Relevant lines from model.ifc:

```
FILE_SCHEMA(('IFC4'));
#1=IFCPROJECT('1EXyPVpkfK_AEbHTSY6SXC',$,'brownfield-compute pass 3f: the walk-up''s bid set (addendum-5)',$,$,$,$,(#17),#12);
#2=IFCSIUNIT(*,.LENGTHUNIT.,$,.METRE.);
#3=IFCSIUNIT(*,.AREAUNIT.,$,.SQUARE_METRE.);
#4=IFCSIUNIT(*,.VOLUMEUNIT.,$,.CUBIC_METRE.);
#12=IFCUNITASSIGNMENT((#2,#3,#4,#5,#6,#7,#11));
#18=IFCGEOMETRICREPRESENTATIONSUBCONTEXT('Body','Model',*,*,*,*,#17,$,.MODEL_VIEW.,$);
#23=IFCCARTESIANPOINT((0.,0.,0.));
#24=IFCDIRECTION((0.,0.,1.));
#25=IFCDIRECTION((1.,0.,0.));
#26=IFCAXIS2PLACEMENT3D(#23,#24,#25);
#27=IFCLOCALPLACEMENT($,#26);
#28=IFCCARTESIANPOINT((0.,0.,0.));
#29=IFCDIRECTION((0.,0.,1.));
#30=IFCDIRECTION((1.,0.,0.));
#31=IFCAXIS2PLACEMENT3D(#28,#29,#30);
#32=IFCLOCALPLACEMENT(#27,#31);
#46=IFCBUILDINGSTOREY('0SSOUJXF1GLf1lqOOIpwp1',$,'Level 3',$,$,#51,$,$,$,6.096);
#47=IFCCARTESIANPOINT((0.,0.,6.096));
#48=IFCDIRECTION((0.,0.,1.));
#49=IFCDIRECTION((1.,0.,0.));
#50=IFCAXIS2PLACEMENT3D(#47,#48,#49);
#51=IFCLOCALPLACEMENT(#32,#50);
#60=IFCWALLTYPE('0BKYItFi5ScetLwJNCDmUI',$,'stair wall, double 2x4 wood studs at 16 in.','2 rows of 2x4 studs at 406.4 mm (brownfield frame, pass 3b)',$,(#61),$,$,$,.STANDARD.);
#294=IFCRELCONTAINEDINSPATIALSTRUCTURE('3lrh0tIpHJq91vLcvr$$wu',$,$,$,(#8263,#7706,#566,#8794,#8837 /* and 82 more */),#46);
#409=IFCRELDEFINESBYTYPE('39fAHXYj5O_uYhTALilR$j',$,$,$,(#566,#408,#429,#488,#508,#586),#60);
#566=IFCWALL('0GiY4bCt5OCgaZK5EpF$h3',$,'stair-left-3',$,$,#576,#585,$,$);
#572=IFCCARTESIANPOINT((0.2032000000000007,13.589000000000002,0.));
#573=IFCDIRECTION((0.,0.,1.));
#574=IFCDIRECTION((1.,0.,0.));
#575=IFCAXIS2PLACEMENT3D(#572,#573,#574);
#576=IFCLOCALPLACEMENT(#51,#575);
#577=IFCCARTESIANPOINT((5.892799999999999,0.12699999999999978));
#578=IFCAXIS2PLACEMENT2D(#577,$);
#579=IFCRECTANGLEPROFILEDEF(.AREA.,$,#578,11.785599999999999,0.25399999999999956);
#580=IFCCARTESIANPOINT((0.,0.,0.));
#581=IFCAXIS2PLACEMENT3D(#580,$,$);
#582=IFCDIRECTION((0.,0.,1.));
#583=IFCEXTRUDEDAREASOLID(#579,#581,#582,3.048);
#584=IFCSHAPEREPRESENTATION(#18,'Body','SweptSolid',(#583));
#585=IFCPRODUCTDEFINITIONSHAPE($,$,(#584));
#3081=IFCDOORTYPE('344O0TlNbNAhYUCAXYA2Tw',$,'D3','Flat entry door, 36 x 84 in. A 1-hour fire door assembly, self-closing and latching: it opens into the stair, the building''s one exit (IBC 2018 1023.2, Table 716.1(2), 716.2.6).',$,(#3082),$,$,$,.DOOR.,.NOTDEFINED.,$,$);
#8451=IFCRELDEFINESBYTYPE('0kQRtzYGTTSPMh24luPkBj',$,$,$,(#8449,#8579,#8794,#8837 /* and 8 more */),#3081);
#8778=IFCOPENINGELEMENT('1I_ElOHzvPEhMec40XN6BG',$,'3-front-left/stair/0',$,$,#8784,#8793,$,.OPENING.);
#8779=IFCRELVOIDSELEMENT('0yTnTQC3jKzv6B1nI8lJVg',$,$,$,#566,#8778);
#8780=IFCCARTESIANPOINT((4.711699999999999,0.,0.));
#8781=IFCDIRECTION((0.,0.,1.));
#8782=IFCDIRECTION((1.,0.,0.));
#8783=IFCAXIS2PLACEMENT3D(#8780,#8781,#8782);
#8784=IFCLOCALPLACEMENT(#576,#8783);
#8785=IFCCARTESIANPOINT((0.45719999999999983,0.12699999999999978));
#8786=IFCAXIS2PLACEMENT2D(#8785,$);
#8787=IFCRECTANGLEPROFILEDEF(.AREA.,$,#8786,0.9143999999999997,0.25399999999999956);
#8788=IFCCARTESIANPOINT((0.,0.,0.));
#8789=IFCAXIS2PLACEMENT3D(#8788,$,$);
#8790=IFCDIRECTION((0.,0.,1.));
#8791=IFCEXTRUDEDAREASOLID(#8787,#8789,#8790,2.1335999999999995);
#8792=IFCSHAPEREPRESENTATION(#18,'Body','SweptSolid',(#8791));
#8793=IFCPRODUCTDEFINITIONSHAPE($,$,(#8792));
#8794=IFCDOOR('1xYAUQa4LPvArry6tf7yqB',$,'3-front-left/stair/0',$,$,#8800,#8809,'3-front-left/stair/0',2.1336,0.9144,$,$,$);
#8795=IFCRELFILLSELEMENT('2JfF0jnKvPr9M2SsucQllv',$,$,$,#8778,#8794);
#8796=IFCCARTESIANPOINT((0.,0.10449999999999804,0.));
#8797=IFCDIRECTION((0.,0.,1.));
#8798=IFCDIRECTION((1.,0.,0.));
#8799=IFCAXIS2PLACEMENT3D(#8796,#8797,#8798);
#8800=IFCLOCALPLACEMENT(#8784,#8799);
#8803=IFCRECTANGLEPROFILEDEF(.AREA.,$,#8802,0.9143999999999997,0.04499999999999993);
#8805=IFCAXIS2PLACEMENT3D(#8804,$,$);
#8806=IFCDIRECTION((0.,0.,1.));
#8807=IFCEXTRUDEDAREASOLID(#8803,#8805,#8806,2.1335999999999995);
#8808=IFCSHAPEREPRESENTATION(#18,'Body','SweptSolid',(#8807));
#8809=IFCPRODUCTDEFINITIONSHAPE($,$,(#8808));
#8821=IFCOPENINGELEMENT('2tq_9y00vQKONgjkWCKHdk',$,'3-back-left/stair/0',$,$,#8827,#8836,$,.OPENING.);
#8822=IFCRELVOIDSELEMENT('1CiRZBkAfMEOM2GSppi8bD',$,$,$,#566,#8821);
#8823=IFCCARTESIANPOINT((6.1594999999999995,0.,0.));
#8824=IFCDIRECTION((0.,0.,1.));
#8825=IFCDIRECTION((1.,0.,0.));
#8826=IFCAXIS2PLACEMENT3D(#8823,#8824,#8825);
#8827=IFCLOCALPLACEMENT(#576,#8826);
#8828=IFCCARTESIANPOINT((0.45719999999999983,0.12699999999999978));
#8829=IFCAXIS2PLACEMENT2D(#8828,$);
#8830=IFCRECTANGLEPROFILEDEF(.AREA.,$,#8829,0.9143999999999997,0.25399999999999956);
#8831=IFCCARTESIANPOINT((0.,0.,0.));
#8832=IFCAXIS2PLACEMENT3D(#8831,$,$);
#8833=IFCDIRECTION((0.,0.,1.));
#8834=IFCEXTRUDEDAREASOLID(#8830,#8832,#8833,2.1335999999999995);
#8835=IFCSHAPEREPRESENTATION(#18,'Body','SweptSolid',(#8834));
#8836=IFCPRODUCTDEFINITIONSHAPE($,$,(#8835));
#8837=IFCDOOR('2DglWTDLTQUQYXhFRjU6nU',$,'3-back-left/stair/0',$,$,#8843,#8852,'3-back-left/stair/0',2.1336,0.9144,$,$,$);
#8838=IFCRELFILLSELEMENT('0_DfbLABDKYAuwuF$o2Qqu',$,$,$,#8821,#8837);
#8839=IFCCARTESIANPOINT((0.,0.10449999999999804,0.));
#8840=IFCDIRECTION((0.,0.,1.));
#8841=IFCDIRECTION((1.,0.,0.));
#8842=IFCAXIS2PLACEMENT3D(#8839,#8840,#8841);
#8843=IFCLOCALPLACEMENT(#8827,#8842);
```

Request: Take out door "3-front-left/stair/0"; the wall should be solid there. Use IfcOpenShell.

```python
import ifcopenshell
import ifcopenshell.api.feature
import ifcopenshell.api.root
import ifcopenshell.geom
import ifcopenshell.util.shape

model = ifcopenshell.open("model.ifc")
settings = ifcopenshell.geom.settings()


def volume(element):
    """Net volume in cubic metres, openings subtracted."""
    shape = ifcopenshell.geom.create_shape(settings, element)
    return ifcopenshell.util.shape.get_volume(shape.geometry)


door = model.by_guid("1xYAUQa4LPvArry6tf7yqB")
opening = door.FillsVoids[0].RelatingOpeningElement
wall = opening.VoidsElements[0].RelatingBuildingElement
before = volume(wall)

ifcopenshell.api.root.remove_product(model, product=door)
ifcopenshell.api.feature.remove_feature(model, feature=opening)

after = volume(wall)

print(f"wall volume {before:.3f} -> {after:.3f} m3")

model.write("model-out.ifc")
```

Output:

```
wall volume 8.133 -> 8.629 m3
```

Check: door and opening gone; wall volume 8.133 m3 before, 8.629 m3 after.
